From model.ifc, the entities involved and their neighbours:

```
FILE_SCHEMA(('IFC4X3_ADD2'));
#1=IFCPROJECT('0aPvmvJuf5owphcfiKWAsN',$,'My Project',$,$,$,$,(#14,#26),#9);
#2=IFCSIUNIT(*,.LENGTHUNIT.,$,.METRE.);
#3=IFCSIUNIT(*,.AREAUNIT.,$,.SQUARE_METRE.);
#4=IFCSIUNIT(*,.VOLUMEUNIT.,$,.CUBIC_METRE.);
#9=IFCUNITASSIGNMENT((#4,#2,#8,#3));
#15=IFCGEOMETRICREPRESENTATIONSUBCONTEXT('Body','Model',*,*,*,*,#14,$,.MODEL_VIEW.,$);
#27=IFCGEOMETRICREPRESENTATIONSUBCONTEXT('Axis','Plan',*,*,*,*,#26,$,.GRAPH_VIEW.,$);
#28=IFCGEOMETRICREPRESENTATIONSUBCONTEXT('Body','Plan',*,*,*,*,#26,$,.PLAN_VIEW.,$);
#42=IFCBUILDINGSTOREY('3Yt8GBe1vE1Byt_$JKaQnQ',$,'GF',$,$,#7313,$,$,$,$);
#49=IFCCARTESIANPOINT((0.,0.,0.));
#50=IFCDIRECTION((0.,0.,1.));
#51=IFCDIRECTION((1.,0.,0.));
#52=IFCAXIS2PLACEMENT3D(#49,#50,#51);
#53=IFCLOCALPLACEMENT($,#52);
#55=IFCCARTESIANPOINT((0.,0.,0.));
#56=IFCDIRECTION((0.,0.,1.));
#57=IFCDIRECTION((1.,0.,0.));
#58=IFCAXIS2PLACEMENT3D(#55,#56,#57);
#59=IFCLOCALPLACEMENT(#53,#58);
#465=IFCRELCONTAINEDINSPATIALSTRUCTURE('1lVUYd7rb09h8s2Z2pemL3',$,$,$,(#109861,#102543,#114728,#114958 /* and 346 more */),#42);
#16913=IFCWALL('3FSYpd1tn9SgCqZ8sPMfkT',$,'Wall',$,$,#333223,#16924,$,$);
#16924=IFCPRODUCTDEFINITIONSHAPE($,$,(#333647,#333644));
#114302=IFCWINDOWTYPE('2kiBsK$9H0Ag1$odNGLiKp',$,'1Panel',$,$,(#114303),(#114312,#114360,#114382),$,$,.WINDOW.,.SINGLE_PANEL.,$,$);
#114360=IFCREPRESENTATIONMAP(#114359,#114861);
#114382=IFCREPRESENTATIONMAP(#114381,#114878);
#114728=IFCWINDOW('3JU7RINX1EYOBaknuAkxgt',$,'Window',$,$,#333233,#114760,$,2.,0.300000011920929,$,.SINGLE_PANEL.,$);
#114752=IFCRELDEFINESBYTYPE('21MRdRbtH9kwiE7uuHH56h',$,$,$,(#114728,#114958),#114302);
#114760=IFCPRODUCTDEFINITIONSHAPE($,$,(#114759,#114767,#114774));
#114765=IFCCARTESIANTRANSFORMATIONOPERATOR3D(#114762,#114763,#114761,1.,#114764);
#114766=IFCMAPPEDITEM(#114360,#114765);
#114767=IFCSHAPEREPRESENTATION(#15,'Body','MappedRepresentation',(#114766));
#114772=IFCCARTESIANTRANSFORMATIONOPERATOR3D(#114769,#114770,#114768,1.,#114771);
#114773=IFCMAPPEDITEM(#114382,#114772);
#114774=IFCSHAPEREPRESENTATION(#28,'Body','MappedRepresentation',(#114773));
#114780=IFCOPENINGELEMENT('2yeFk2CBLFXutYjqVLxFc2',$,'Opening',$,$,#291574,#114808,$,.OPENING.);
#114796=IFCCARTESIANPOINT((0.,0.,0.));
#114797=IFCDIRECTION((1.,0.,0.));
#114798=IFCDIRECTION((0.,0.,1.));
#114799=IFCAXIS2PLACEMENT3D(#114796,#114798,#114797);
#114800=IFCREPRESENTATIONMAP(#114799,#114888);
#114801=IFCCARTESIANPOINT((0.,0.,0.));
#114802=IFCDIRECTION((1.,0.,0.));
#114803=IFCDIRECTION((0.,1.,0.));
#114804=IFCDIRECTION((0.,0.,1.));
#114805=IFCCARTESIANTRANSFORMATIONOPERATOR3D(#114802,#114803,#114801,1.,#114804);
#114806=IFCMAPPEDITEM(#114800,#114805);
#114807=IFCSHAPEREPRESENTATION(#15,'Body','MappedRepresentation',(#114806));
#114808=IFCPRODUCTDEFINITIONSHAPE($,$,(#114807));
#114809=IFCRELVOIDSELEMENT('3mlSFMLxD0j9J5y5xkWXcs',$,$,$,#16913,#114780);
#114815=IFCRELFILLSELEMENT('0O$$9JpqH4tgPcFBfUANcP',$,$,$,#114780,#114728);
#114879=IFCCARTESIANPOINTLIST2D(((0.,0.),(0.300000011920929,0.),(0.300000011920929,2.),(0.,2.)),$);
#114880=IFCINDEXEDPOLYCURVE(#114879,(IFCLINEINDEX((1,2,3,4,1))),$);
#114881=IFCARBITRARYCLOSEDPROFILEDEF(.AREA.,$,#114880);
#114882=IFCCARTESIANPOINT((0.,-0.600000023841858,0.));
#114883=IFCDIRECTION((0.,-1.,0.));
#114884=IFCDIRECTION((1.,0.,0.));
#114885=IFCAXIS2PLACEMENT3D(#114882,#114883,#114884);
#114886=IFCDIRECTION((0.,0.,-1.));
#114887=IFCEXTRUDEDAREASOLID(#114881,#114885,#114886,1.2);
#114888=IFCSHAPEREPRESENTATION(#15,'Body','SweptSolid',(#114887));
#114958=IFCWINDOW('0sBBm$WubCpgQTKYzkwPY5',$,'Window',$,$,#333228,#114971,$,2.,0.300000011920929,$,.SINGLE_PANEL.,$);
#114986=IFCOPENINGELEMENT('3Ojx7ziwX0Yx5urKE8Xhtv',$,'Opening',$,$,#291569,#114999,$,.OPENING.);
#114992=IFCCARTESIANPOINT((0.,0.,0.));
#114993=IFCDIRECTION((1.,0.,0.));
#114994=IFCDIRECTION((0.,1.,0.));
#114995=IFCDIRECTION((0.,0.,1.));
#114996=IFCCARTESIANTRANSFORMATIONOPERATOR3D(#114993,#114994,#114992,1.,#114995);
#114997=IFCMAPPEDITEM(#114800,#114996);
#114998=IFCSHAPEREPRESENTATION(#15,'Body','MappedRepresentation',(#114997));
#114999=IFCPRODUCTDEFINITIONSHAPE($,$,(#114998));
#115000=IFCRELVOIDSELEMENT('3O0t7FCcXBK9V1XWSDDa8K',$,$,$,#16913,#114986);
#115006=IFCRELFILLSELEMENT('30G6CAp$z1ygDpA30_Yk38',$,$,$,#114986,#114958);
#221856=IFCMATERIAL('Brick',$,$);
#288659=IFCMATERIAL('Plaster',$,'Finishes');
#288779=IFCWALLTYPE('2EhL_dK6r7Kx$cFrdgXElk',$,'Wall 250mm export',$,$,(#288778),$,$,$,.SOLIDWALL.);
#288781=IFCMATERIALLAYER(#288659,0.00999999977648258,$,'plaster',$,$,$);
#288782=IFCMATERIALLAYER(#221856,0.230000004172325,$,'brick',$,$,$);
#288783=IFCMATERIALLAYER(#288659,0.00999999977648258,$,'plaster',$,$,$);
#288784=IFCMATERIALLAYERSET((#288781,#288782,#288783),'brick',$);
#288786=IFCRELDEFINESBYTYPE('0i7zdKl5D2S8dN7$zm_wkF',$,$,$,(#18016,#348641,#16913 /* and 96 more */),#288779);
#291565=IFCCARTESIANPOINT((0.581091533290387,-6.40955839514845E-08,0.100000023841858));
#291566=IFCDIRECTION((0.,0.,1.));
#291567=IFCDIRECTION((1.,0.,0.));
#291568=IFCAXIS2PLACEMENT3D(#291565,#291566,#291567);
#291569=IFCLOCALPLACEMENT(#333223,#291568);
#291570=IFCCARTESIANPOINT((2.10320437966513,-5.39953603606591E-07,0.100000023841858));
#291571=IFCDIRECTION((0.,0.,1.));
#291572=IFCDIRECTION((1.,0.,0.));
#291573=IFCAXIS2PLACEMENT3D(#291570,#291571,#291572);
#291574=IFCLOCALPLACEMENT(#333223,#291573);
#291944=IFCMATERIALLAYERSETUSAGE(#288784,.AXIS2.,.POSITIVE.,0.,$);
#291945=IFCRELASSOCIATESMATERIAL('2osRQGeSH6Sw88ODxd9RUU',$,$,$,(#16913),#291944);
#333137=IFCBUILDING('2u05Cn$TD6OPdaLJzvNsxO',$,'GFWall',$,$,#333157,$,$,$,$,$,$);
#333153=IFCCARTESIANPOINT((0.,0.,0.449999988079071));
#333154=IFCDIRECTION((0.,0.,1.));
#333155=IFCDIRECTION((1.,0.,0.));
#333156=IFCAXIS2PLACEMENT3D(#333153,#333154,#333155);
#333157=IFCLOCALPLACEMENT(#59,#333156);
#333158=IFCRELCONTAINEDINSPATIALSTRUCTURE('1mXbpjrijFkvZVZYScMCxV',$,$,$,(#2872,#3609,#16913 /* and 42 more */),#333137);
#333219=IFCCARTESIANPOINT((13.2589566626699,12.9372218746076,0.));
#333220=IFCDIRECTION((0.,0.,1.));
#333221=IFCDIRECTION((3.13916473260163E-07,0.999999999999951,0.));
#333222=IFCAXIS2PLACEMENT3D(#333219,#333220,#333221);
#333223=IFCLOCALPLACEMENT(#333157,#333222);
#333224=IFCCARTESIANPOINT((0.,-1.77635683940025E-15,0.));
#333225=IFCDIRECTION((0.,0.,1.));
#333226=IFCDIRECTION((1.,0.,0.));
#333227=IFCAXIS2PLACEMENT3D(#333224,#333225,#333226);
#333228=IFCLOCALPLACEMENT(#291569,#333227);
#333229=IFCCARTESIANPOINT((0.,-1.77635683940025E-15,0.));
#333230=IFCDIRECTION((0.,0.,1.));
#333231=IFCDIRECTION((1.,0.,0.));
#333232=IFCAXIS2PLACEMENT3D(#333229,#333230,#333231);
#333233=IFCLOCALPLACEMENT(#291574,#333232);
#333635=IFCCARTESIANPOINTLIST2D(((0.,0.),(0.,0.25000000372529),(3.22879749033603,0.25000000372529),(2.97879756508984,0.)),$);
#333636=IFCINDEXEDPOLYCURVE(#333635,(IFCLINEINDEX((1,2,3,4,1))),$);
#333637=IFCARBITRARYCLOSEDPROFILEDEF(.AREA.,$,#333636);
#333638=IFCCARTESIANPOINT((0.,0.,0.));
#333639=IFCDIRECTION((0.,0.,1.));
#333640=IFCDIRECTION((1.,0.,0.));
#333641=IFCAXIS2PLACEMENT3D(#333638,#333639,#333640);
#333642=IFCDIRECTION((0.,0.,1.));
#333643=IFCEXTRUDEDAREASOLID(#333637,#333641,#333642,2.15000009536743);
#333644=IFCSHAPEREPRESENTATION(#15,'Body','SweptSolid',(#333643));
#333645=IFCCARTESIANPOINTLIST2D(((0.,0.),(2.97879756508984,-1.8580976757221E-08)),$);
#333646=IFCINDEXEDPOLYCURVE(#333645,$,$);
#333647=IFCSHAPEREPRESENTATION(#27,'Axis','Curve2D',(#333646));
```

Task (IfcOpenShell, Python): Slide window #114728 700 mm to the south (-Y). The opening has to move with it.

```python
import ifcopenshell
import ifcopenshell.api.geometry
import ifcopenshell.util.placement

model = ifcopenshell.open("model.ifc")

window = model.by_guid("3JU7RINX1EYOBaknuAkxgt")
opening = window.FillsVoids[0].RelatingOpeningElement
wall = opening.VoidsElements[0].RelatingBuildingElement

wall_matrix = ifcopenshell.util.placement.get_local_placement(wall.ObjectPlacement)
shift = wall_matrix[:3, 0] * -0.7
before = ifcopenshell.util.placement.get_local_placement(window.ObjectPlacement)[:3, 3].copy()

# The window is placed relative to its opening, so it follows when the opening moves.
matrix = ifcopenshell.util.placement.get_local_placement(opening.ObjectPlacement)
matrix[:3, 3] += shift
ifcopenshell.api.geometry.edit_object_placement(
    model, product=opening, matrix=matrix, is_si=False, should_transform_children=True
)

after = ifcopenshell.util.placement.get_local_placement(window.ObjectPlacement)[:3, 3]
print("window moved by", (after - before).round(3) + 0.0)

model.write("model_rev.ifc")
```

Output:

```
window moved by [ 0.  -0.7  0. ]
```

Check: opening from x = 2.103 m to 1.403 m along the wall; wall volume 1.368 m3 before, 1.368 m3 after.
